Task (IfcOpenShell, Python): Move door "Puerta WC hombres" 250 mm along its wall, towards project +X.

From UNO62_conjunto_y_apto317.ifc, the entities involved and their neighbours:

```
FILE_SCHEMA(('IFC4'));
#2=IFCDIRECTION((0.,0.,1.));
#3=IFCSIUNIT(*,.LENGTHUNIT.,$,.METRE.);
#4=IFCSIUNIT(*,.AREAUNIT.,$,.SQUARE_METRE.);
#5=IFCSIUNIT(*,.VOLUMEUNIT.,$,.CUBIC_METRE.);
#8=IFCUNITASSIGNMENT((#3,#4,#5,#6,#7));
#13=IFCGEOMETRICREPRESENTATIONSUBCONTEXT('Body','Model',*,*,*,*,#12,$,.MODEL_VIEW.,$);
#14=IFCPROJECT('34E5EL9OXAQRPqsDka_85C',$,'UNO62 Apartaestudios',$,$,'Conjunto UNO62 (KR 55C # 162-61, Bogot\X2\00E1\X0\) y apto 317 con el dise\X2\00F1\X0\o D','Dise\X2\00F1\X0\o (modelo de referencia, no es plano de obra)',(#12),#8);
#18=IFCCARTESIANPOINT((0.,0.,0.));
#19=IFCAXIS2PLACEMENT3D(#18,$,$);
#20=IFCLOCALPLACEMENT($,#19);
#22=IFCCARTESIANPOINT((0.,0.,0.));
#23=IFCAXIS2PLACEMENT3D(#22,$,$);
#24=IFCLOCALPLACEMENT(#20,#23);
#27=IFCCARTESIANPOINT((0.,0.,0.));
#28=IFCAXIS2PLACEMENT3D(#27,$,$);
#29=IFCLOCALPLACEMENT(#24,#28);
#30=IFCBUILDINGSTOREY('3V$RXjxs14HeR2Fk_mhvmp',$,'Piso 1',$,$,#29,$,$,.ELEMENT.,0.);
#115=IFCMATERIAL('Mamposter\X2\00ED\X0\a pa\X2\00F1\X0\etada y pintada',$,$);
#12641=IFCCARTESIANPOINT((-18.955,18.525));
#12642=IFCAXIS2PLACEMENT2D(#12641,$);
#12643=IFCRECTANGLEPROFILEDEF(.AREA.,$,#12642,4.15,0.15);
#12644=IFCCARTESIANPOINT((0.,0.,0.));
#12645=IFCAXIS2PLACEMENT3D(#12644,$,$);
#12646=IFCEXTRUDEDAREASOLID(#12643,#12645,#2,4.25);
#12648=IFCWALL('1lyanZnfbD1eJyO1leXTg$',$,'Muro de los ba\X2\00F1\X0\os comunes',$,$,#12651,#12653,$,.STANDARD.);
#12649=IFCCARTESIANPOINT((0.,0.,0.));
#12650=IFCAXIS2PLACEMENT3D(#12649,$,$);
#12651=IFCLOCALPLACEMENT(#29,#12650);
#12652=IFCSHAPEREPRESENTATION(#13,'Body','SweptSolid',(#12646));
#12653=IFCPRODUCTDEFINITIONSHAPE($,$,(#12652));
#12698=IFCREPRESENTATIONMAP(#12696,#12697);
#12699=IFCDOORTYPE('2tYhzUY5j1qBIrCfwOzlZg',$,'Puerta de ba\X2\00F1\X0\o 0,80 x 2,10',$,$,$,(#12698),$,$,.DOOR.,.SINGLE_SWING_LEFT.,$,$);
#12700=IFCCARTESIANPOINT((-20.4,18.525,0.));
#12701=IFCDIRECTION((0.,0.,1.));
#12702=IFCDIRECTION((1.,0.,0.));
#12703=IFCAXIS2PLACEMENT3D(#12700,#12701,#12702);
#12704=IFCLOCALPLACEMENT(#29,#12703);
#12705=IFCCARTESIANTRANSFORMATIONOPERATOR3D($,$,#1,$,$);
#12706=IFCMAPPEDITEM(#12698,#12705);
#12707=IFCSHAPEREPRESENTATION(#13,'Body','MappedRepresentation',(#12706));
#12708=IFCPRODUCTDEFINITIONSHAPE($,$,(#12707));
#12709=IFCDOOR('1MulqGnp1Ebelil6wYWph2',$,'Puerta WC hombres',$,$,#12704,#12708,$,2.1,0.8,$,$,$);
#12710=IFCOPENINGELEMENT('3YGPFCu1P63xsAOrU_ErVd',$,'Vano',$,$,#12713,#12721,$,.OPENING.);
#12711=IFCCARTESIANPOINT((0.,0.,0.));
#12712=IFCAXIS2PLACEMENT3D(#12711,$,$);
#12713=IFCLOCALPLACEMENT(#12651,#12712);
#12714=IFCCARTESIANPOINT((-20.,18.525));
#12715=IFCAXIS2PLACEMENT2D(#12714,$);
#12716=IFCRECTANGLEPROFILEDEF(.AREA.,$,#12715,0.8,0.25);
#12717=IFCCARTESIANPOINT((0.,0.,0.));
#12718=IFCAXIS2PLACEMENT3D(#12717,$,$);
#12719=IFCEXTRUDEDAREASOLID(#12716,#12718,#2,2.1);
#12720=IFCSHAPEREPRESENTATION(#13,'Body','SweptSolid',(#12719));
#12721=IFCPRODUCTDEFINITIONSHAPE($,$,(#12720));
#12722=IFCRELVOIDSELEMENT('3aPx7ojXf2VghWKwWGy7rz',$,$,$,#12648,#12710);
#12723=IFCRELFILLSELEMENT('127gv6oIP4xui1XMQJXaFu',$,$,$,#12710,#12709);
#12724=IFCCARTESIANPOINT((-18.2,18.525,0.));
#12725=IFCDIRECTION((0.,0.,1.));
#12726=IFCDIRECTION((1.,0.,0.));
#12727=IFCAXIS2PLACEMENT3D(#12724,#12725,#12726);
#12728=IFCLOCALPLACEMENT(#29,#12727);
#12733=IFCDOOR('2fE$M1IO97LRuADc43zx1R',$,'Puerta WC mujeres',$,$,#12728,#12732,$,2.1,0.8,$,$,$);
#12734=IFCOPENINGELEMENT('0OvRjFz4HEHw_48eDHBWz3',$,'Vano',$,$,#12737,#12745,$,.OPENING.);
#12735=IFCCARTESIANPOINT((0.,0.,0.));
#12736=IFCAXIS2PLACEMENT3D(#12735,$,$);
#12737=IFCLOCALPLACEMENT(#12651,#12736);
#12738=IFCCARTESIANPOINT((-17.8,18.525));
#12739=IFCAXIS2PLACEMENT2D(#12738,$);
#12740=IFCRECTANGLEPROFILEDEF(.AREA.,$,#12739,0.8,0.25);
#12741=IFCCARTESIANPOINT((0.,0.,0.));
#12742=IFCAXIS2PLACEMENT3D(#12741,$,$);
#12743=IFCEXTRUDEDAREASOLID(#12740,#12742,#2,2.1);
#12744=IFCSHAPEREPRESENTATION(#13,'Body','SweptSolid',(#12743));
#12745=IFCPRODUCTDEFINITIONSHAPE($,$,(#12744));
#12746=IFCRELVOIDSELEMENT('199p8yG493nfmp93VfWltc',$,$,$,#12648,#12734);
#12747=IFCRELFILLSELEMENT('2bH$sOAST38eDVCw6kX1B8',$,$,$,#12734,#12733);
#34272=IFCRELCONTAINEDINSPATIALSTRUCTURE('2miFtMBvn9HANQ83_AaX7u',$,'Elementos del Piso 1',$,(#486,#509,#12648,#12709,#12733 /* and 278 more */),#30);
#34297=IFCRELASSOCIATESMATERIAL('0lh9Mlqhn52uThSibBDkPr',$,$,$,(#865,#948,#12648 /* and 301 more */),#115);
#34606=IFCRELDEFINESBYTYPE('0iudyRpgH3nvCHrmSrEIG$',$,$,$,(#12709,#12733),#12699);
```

```python
import ifcopenshell
import ifcopenshell.api.geometry
import ifcopenshell.util.placement
import ifcopenshell.util.unit

model = ifcopenshell.open("UNO62_conjunto_y_apto317.ifc")
unit_scale = ifcopenshell.util.unit.calculate_unit_scale(model)

door = model.by_guid("1MulqGnp1Ebelil6wYWph2")
opening = door.FillsVoids[0].RelatingOpeningElement
wall = opening.VoidsElements[0].RelatingBuildingElement

wall_matrix = ifcopenshell.util.placement.get_local_placement(wall.ObjectPlacement)
shift = wall_matrix[:3, 0] * 0.25 / unit_scale
before = ifcopenshell.util.placement.get_local_placement(door.ObjectPlacement)[:3, 3].copy()

# The door is not placed relative to its opening, so move both.
for product in (opening, door):
    matrix = ifcopenshell.util.placement.get_local_placement(product.ObjectPlacement)
    matrix[:3, 3] += shift
    ifcopenshell.api.geometry.edit_object_placement(model, product=product, matrix=matrix, is_si=False)

after = ifcopenshell.util.placement.get_local_placement(door.ObjectPlacement)[:3, 3]
print("door moved by", (after - before).round(3) + 0.0)

model.write("UNO62_conjunto_y_apto317-out.ifc")
```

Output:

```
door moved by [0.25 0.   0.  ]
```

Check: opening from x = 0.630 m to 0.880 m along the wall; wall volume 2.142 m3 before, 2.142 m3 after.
